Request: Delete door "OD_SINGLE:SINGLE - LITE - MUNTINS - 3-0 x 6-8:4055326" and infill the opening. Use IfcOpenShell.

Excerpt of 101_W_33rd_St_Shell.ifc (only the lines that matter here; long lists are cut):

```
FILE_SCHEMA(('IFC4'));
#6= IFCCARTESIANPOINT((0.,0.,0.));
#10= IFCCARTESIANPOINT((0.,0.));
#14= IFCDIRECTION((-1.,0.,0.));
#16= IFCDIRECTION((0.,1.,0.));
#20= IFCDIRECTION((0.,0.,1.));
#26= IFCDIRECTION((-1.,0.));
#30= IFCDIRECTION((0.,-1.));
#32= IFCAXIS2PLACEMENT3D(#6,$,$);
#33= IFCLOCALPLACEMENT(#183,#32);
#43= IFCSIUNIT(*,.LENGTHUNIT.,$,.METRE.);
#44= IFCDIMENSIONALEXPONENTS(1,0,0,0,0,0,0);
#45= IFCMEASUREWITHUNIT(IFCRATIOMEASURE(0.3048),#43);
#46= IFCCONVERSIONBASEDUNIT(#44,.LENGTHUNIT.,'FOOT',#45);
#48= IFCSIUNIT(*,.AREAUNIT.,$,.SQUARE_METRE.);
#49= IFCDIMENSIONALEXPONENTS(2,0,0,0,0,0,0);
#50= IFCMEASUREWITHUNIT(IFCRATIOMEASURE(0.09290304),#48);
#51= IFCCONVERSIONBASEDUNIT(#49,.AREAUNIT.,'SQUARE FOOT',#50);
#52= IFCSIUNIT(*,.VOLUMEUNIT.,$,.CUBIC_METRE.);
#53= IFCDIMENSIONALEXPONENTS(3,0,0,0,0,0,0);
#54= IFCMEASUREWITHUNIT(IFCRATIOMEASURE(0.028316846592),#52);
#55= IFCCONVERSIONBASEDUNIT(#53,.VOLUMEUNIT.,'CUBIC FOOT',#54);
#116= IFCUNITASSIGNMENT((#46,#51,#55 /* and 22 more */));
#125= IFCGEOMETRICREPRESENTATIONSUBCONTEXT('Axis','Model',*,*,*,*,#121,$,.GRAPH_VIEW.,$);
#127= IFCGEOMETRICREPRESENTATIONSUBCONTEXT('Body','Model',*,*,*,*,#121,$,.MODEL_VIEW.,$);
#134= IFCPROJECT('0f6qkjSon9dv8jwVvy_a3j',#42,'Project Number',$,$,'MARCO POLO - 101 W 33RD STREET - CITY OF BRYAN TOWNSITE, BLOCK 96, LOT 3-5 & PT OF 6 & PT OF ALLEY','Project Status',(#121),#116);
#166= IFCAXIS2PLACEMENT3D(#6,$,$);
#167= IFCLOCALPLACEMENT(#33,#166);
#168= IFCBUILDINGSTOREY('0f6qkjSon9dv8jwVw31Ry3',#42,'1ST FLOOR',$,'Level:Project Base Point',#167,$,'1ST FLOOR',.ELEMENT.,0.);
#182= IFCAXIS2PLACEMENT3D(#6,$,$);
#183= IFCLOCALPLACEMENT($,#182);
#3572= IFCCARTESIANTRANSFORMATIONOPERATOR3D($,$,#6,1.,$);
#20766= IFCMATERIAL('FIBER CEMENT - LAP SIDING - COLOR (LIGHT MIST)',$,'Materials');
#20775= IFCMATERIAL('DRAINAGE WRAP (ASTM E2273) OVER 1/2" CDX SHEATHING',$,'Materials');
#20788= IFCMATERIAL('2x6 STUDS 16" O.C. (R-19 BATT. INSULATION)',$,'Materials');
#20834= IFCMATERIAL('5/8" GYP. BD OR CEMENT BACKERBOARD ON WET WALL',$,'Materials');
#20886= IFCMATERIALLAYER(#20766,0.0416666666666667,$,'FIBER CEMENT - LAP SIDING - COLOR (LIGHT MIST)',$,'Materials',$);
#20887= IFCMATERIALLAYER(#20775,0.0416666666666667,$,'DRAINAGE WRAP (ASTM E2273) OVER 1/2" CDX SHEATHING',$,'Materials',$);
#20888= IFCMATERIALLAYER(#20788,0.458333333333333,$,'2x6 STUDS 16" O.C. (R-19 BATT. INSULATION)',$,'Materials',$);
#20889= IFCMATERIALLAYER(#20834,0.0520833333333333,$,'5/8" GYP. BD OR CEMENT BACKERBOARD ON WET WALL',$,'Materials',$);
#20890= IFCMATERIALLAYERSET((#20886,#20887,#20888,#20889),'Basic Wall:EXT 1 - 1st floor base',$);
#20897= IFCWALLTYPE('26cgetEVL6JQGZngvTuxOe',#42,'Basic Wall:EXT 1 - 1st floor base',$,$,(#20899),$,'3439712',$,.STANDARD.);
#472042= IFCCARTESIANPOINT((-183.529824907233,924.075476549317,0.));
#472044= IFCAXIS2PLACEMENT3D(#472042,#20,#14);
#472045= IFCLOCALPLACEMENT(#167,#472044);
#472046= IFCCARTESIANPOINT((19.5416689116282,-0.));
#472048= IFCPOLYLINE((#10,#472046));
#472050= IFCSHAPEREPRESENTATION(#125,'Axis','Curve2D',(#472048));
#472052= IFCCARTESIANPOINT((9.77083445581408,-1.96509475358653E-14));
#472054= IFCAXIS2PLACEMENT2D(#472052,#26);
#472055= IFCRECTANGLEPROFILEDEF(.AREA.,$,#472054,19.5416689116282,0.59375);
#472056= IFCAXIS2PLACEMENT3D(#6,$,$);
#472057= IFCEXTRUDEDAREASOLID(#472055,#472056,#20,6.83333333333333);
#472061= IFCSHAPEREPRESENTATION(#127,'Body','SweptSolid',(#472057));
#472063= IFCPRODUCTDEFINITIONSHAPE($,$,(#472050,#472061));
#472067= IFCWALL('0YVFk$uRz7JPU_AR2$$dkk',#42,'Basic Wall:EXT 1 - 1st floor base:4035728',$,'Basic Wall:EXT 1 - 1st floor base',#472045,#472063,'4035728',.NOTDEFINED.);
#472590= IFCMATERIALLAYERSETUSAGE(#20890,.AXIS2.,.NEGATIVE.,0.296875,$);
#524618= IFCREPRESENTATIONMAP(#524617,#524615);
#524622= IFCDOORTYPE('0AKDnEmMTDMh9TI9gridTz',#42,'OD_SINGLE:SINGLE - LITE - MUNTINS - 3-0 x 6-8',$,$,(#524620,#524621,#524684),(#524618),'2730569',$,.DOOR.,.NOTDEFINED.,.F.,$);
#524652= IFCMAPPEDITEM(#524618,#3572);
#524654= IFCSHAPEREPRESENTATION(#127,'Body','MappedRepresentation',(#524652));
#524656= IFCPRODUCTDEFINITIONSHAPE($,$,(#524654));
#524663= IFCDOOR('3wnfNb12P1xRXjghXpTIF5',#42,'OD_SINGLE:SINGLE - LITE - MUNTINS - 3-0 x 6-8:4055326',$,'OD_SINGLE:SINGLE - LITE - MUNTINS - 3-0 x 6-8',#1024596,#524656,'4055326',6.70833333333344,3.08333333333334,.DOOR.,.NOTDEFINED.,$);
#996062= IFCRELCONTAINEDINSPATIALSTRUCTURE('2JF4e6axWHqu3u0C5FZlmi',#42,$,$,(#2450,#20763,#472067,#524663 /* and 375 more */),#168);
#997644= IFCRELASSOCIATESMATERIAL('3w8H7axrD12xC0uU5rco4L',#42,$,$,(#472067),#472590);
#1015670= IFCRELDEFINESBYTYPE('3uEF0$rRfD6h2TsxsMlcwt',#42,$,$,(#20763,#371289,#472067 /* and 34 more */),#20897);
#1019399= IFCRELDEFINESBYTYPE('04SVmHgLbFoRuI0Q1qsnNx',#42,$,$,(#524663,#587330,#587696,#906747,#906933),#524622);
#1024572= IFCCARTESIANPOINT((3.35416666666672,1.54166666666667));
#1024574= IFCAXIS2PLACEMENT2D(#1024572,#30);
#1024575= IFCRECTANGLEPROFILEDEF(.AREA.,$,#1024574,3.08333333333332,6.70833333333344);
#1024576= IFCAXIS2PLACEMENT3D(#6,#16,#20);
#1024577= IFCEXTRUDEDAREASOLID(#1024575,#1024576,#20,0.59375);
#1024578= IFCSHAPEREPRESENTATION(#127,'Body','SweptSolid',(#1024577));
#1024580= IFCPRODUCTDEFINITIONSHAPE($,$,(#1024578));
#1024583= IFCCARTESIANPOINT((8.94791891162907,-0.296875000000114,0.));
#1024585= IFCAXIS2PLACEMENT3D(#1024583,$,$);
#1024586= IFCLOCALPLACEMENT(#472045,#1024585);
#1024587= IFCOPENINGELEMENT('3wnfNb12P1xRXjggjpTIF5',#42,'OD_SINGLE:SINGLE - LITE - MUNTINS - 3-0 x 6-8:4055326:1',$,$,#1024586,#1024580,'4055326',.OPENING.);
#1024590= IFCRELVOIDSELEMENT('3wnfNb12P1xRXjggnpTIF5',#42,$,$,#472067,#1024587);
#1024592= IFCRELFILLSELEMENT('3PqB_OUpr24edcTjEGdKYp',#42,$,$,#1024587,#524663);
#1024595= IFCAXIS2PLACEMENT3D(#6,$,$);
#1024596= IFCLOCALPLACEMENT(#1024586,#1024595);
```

```python
import ifcopenshell
import ifcopenshell.api.feature
import ifcopenshell.api.root
import ifcopenshell.geom
import ifcopenshell.util.shape

model = ifcopenshell.open("101_W_33rd_St_Shell.ifc")
settings = ifcopenshell.geom.settings()


def volume(element):
    """Net volume in cubic metres, openings subtracted."""
    shape = ifcopenshell.geom.create_shape(settings, element)
    return ifcopenshell.util.shape.get_volume(shape.geometry)


door = model.by_id(524663)
opening = door.FillsVoids[0].RelatingOpeningElement
wall = opening.VoidsElements[0].RelatingBuildingElement
before = volume(wall)

ifcopenshell.api.root.remove_product(model, product=door)
ifcopenshell.api.feature.remove_feature(model, feature=opening)

after = volume(wall)

print(f"wall volume {before:.3f} -> {after:.3f} m3")

model.write("101_W_33rd_St_Shell_rev.ifc")
```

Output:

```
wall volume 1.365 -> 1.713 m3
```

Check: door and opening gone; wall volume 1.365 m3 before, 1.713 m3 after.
